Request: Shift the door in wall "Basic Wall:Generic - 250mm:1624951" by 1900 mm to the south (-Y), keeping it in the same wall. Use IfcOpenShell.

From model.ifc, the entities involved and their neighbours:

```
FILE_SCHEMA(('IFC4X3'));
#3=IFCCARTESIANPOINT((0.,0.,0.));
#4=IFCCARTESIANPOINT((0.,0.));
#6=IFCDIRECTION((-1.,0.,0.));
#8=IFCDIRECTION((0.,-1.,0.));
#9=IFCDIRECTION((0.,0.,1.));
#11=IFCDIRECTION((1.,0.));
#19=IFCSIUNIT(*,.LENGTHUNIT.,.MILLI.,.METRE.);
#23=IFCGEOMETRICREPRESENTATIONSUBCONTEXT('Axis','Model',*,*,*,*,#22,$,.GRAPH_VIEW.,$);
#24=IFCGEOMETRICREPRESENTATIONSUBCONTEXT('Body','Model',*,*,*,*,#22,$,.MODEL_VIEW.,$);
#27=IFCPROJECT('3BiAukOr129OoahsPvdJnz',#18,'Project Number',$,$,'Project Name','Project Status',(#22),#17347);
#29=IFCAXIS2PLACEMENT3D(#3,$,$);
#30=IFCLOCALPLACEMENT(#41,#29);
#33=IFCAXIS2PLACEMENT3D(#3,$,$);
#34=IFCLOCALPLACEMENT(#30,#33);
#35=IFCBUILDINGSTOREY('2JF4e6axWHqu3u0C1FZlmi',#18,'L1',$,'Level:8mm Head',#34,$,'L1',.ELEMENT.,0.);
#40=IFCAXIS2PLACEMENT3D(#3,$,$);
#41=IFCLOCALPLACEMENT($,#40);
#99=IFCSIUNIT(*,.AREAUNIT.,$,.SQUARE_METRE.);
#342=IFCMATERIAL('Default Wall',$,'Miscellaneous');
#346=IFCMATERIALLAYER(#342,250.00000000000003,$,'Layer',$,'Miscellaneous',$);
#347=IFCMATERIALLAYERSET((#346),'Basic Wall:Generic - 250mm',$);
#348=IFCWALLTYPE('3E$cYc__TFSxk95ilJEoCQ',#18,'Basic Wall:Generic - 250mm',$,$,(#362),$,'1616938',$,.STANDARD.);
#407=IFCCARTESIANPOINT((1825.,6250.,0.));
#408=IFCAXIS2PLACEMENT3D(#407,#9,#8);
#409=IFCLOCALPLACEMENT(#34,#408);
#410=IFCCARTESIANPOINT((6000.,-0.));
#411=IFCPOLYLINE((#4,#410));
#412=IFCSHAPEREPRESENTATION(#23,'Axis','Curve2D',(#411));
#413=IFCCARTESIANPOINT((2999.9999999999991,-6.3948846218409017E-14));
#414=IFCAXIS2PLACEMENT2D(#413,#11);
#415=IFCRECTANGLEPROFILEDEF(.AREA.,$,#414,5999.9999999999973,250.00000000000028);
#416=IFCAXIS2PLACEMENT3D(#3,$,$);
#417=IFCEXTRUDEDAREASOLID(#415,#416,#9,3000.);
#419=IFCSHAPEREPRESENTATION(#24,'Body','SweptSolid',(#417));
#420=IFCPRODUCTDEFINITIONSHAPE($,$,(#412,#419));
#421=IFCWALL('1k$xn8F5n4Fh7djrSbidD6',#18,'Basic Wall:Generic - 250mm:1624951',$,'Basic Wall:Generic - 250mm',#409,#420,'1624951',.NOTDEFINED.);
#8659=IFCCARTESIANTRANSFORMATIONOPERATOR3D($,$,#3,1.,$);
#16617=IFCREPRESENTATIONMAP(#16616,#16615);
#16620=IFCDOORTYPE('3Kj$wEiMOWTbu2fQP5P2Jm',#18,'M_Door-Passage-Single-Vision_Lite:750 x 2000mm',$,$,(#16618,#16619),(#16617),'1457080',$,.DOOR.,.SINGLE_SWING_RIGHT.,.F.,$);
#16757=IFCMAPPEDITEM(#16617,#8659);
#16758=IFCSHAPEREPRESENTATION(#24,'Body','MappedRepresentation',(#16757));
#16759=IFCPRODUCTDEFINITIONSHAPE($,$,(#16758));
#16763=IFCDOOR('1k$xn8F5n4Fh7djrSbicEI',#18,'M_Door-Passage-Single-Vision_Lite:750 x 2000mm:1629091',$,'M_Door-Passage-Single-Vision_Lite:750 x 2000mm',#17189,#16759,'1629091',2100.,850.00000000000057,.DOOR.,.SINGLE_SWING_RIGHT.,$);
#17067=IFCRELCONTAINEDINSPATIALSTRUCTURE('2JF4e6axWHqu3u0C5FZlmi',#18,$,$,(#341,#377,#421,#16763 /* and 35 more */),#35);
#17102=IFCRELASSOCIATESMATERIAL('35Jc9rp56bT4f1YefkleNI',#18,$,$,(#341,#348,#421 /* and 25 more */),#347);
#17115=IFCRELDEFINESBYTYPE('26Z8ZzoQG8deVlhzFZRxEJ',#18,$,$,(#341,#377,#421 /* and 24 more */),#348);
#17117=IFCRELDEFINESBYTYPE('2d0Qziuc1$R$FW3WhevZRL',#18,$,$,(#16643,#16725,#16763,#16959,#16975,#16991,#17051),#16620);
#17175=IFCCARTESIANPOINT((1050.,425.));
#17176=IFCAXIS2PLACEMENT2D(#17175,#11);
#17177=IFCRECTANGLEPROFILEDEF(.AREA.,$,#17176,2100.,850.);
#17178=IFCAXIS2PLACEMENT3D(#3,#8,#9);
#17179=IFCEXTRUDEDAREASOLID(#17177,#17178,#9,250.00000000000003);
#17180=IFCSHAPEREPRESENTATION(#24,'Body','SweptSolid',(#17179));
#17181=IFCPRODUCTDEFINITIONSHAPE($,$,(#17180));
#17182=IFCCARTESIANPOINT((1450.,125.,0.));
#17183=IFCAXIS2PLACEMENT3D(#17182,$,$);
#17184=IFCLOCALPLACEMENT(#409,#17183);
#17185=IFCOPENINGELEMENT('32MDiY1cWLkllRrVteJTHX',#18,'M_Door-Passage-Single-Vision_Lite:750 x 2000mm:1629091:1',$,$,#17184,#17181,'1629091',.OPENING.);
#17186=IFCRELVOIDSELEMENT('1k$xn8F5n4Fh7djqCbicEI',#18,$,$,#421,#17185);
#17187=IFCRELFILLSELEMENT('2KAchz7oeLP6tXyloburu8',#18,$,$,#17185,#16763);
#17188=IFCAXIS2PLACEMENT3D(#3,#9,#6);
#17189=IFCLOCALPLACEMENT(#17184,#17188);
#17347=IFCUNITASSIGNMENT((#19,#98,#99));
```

```python
import ifcopenshell
import ifcopenshell.api.geometry
import ifcopenshell.util.placement
import ifcopenshell.util.unit

model = ifcopenshell.open("model.ifc")
unit_scale = ifcopenshell.util.unit.calculate_unit_scale(model)

door = model.by_id(16763)
opening = door.FillsVoids[0].RelatingOpeningElement
wall = opening.VoidsElements[0].RelatingBuildingElement

wall_matrix = ifcopenshell.util.placement.get_local_placement(wall.ObjectPlacement)
shift = wall_matrix[:3, 0] * 1.9 / unit_scale
before = ifcopenshell.util.placement.get_local_placement(door.ObjectPlacement)[:3, 3].copy()

# The door is placed relative to its opening, so it follows when the opening moves.
matrix = ifcopenshell.util.placement.get_local_placement(opening.ObjectPlacement)
matrix[:3, 3] += shift
ifcopenshell.api.geometry.edit_object_placement(
    model, product=opening, matrix=matrix, is_si=False, should_transform_children=True
)

after = ifcopenshell.util.placement.get_local_placement(door.ObjectPlacement)[:3, 3]
print("door moved by", (after - before).round(3) + 0.0)

model.write("model-out.ifc")
```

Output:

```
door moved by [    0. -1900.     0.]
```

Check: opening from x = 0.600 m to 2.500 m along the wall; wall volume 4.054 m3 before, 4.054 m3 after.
